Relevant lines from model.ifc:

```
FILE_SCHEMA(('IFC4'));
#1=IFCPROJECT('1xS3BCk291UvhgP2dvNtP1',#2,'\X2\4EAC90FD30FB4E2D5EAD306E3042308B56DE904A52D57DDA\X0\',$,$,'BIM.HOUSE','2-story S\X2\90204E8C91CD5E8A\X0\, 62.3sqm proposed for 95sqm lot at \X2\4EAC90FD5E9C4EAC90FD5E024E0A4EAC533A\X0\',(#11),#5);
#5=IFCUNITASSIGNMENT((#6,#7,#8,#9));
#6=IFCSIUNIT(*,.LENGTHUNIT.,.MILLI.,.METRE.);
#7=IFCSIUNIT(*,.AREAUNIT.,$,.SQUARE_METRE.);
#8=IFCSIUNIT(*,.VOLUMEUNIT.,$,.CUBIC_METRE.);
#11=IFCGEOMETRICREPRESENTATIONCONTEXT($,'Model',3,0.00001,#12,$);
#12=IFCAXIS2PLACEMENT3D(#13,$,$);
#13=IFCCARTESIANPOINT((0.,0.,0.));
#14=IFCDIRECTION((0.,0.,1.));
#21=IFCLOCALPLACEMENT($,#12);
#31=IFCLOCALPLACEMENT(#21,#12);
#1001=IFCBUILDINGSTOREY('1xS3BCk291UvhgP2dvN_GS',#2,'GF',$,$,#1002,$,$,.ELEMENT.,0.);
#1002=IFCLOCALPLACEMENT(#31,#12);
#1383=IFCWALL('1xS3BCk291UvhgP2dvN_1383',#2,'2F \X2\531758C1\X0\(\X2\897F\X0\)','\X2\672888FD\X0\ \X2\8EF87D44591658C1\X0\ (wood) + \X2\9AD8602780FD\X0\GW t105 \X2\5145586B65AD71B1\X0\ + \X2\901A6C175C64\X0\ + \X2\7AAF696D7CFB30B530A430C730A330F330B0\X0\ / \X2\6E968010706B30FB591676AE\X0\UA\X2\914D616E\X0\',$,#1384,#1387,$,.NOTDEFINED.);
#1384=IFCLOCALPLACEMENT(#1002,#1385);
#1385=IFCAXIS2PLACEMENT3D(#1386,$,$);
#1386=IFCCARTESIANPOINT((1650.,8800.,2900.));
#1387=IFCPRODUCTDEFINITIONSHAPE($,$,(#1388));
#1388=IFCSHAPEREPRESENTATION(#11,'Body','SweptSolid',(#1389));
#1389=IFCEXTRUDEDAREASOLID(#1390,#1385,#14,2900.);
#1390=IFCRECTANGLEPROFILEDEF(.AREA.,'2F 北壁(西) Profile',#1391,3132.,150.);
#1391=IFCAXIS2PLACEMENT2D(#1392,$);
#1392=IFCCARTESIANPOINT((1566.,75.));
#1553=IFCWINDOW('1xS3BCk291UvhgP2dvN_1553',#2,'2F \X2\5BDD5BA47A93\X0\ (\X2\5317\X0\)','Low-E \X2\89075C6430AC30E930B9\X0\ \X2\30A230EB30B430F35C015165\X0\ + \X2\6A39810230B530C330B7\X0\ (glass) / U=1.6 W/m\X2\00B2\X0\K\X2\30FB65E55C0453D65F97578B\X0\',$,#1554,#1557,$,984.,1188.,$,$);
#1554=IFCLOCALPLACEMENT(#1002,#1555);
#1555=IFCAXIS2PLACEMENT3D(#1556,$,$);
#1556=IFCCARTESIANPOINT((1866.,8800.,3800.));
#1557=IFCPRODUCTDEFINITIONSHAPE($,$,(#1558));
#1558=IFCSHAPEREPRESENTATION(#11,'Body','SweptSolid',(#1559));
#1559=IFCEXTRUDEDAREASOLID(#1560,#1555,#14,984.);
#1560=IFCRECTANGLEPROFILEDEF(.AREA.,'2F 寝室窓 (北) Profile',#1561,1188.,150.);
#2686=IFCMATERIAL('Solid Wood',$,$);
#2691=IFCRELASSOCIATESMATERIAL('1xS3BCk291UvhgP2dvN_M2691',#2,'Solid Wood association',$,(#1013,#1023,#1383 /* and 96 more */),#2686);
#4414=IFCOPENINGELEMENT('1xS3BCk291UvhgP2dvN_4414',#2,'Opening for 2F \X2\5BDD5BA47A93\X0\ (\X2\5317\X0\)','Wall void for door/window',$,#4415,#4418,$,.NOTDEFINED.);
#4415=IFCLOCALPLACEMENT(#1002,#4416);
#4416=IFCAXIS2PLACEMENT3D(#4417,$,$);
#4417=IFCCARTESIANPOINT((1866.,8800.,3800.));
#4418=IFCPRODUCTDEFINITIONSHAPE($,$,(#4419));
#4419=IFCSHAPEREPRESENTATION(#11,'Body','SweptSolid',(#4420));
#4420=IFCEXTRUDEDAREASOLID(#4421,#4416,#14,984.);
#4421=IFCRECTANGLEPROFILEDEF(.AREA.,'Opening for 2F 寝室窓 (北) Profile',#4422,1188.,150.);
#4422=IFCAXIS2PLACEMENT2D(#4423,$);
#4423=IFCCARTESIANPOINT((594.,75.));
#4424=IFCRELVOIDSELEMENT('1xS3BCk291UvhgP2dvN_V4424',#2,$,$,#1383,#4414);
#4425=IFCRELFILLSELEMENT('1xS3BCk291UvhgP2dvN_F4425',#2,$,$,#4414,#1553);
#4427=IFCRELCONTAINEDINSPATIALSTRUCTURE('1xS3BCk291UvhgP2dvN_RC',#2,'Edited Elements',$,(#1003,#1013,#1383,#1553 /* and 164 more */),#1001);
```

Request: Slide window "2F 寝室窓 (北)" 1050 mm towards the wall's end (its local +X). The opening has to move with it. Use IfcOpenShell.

```python
import ifcopenshell
import ifcopenshell.api.geometry
import ifcopenshell.util.placement

model = ifcopenshell.open("model.ifc")

window = model.by_guid("1xS3BCk291UvhgP2dvN_1553")
opening = window.FillsVoids[0].RelatingOpeningElement
wall = opening.VoidsElements[0].RelatingBuildingElement

wall_matrix = ifcopenshell.util.placement.get_local_placement(wall.ObjectPlacement)
shift = wall_matrix[:3, 0] * 1050.0
before = ifcopenshell.util.placement.get_local_placement(window.ObjectPlacement)[:3, 3].copy()

# The window is not placed relative to its opening, so move both.
for product in (opening, window):
    matrix = ifcopenshell.util.placement.get_local_placement(product.ObjectPlacement)
    matrix[:3, 3] += shift
    ifcopenshell.api.geometry.edit_object_placement(model, product=product, matrix=matrix, is_si=False)

after = ifcopenshell.util.placement.get_local_placement(window.ObjectPlacement)[:3, 3]
print("window moved by", (after - before).round(3) + 0.0)

model.write("model_edited.ifc")
```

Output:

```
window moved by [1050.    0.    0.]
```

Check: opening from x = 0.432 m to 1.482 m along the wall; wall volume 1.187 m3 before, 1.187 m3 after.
